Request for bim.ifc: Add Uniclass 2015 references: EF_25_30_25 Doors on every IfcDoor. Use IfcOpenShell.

First a look at what the model holds.

```python
import ifcopenshell

model = ifcopenshell.open("bim.ifc")
print(model.schema)
print("classifications:", [c.Name for c in model.by_type("IfcClassification")])
for ifc_class in ("IfcDoor", "IfcRoof", "IfcStair", "IfcWall", "IfcWindow"):
    print(ifc_class, len(model.by_type(ifc_class)))
```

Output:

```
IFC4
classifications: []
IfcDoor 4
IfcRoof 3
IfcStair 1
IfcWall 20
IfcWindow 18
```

```python
import ifcopenshell
import ifcopenshell.api.classification

model = ifcopenshell.open("bim.ifc")

system = ifcopenshell.api.classification.add_classification(model, classification="Uniclass 2015")

codes = {
    "IfcDoor": ("EF_25_30_25", "Doors"),
}
for ifc_class, (code, name) in codes.items():
    products = model.by_type(ifc_class)
    ifcopenshell.api.classification.add_reference(
        model, products=products, classification=system, identification=code, name=name
    )
    print(code, len(products))

model.write("bim_v2.ifc")
```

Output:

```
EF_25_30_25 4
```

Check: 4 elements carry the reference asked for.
